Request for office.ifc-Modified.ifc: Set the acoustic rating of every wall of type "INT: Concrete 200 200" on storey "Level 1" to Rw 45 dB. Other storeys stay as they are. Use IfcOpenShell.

First a look at what the model holds.

```python
import ifcopenshell
import ifcopenshell.util.element

model = ifcopenshell.open("office.ifc-Modified.ifc")
print(model.schema)
storey = next(s for s in model.by_type("IfcBuildingStorey") if s.Name == "Level 1")
walls = [e for e in ifcopenshell.util.element.get_decomposition(storey) if e.is_a("IfcWall")]
seen = {}
for e in walls:
    element_type = ifcopenshell.util.element.get_type(e)
    key = (element_type.Name if element_type != e and element_type else None, ifcopenshell.util.element.get_pset(e, "Pset_WallCommon", "AcousticRating"))
    seen[key] = seen.get(key, 0) + 1
for (name, value), count in sorted(seen.items(), key=str):
    print(count, "x", name, "|", value)
```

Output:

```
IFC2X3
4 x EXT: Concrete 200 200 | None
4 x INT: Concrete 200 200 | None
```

```python
import ifcopenshell
import ifcopenshell.api.pset
import ifcopenshell.util.element

model = ifcopenshell.open("office.ifc-Modified.ifc")

storey = next(s for s in model.by_type("IfcBuildingStorey") if s.Name == "Level 1")
walls = [e for e in ifcopenshell.util.element.get_decomposition(storey) if e.is_a("IfcWall")]

count = 0
for e in walls:
    element_type = ifcopenshell.util.element.get_type(e)
    if element_type in (None, e) or element_type.Name != "INT: Concrete 200 200":
        continue
    # add_pset returns the element's existing set when there is one.
    pset = ifcopenshell.api.pset.add_pset(model, product=e, name="Pset_WallCommon")
    ifcopenshell.api.pset.edit_pset(model, pset=pset, properties={"AcousticRating": "Rw 45 dB"})
    count += 1

print(count, "walls updated")

model.write("office.ifc-Modified-out.ifc")
```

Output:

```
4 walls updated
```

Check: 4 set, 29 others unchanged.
